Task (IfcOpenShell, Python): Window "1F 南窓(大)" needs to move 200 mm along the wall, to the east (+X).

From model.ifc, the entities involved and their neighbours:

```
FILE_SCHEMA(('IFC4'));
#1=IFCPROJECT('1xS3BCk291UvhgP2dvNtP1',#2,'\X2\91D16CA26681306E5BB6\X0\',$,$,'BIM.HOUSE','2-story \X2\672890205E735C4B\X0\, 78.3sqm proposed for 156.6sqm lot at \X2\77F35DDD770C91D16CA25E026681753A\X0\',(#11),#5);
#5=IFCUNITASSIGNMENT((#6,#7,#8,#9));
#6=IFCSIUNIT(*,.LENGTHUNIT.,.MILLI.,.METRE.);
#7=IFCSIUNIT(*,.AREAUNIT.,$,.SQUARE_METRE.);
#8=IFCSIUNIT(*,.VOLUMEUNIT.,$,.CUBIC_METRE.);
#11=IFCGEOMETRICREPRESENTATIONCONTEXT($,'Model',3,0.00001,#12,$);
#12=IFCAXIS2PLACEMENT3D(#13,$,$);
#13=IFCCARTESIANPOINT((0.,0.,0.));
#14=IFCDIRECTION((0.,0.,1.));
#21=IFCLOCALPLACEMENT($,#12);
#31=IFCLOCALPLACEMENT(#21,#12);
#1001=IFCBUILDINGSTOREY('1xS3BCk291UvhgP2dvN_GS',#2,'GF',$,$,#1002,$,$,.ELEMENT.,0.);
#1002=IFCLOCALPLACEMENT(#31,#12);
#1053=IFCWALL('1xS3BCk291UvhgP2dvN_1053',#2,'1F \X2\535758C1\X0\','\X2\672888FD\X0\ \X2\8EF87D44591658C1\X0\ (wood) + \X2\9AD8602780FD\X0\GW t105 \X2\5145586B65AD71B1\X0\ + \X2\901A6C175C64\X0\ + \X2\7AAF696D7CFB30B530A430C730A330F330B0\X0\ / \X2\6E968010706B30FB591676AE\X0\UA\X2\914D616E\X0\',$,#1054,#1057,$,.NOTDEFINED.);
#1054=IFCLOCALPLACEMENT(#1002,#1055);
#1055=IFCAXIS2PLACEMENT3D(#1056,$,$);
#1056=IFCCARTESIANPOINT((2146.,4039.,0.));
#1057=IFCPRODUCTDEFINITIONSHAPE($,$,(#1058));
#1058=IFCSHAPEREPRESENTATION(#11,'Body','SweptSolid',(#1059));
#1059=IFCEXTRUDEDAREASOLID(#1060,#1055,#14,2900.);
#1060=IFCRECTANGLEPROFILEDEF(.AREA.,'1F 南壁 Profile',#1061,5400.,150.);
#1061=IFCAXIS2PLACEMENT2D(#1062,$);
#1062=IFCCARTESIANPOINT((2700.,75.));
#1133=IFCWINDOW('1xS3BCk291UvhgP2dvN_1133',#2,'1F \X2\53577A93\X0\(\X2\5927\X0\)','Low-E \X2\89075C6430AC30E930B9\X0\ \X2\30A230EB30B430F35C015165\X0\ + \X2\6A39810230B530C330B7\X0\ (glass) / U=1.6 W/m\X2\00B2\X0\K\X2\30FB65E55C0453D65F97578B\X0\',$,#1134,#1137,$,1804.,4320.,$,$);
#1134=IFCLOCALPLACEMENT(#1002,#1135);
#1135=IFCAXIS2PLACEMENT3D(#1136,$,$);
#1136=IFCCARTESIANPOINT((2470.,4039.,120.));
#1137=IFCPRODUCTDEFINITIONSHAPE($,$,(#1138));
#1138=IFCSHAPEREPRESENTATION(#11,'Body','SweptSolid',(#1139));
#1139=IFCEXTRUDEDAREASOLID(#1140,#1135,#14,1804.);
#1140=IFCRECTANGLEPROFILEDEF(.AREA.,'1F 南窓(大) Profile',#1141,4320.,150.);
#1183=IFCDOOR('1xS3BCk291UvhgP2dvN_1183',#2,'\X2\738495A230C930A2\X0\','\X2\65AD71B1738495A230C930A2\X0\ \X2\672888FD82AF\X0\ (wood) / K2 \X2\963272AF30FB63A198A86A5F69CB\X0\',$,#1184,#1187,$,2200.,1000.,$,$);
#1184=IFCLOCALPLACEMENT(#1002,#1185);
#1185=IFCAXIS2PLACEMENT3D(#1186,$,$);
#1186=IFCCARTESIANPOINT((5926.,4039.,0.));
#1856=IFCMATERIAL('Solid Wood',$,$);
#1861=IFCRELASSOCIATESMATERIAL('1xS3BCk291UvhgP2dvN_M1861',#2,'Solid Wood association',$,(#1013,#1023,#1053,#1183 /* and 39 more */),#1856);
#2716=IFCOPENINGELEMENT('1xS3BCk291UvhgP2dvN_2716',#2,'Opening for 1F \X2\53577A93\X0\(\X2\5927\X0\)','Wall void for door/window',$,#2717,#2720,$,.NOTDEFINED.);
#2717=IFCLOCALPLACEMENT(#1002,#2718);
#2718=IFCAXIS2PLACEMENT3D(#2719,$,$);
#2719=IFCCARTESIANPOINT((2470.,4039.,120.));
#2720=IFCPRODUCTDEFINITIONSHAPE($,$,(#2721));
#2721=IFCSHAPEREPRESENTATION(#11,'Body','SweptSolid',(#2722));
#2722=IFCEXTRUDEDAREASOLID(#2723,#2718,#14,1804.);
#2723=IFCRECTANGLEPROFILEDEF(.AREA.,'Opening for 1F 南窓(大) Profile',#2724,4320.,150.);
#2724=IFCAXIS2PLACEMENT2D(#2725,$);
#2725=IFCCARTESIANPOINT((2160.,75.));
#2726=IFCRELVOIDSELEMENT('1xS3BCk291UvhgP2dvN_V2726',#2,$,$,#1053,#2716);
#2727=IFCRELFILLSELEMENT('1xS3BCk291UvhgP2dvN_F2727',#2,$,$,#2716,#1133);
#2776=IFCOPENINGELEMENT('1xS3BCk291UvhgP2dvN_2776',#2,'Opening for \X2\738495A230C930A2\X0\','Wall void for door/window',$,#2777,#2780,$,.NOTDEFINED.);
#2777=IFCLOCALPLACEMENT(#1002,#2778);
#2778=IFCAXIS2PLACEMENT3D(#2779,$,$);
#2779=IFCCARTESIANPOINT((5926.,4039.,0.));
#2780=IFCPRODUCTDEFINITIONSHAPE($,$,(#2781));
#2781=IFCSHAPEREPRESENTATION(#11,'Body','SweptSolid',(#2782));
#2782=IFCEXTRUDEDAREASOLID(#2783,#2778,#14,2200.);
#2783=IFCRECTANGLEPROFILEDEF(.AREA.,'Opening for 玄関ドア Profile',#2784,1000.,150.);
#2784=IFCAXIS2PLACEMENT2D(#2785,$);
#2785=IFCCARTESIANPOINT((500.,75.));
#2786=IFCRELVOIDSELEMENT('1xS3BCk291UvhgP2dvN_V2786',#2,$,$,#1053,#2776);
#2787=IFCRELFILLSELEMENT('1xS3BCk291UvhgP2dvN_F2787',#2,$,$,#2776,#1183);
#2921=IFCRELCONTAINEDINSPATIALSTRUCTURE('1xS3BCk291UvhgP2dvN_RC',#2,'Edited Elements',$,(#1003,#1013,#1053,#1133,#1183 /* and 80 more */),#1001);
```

```python
import ifcopenshell
import ifcopenshell.api.geometry
import ifcopenshell.util.placement
import ifcopenshell.util.unit

model = ifcopenshell.open("model.ifc")
unit_scale = ifcopenshell.util.unit.calculate_unit_scale(model)

window = model.by_id(1133)
opening = window.FillsVoids[0].RelatingOpeningElement
wall = opening.VoidsElements[0].RelatingBuildingElement

wall_matrix = ifcopenshell.util.placement.get_local_placement(wall.ObjectPlacement)
shift = wall_matrix[:3, 0] * 0.2 / unit_scale
before = ifcopenshell.util.placement.get_local_placement(window.ObjectPlacement)[:3, 3].copy()

# The window is not placed relative to its opening, so move both.
for product in (opening, window):
    matrix = ifcopenshell.util.placement.get_local_placement(product.ObjectPlacement)
    matrix[:3, 3] += shift
    ifcopenshell.api.geometry.edit_object_placement(model, product=product, matrix=matrix, is_si=False)

after = ifcopenshell.util.placement.get_local_placement(window.ObjectPlacement)[:3, 3]
print("window moved by", (after - before).round(3) + 0.0)

model.write("model_updated.ifc")
```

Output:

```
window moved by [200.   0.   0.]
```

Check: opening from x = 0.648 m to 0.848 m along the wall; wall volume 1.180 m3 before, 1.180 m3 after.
